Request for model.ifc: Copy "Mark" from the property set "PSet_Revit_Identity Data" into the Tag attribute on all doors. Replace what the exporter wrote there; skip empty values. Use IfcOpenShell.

First a look at what the model holds.

```python
import ifcopenshell
import ifcopenshell.util.element

model = ifcopenshell.open("model.ifc")
print(model.schema)
doors = model.by_type("IfcDoor")
print(len(doors), "doors")
for e in doors[:8]:
    source = ifcopenshell.util.element.get_pset(e, "PSet_Revit_Identity Data", "Mark")
    target = e.Tag
    print(e.id(), repr(source), repr(target), sep=" | ")
```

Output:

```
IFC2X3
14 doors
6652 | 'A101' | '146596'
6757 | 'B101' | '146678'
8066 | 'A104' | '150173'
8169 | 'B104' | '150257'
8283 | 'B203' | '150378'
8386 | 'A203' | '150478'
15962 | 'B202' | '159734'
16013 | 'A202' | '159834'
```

```python
import ifcopenshell
import ifcopenshell.util.element

model = ifcopenshell.open("model.ifc")

count = 0
for e in model.by_type("IfcDoor"):
    value = ifcopenshell.util.element.get_pset(e, "PSet_Revit_Identity Data", "Mark")
    current = e.Tag
    if not value or not value.strip() or current == value:
        continue
    e.Tag = value
    count += 1

print(count, "doors updated")

model.write("model_v2.ifc")
```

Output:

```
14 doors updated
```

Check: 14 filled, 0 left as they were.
